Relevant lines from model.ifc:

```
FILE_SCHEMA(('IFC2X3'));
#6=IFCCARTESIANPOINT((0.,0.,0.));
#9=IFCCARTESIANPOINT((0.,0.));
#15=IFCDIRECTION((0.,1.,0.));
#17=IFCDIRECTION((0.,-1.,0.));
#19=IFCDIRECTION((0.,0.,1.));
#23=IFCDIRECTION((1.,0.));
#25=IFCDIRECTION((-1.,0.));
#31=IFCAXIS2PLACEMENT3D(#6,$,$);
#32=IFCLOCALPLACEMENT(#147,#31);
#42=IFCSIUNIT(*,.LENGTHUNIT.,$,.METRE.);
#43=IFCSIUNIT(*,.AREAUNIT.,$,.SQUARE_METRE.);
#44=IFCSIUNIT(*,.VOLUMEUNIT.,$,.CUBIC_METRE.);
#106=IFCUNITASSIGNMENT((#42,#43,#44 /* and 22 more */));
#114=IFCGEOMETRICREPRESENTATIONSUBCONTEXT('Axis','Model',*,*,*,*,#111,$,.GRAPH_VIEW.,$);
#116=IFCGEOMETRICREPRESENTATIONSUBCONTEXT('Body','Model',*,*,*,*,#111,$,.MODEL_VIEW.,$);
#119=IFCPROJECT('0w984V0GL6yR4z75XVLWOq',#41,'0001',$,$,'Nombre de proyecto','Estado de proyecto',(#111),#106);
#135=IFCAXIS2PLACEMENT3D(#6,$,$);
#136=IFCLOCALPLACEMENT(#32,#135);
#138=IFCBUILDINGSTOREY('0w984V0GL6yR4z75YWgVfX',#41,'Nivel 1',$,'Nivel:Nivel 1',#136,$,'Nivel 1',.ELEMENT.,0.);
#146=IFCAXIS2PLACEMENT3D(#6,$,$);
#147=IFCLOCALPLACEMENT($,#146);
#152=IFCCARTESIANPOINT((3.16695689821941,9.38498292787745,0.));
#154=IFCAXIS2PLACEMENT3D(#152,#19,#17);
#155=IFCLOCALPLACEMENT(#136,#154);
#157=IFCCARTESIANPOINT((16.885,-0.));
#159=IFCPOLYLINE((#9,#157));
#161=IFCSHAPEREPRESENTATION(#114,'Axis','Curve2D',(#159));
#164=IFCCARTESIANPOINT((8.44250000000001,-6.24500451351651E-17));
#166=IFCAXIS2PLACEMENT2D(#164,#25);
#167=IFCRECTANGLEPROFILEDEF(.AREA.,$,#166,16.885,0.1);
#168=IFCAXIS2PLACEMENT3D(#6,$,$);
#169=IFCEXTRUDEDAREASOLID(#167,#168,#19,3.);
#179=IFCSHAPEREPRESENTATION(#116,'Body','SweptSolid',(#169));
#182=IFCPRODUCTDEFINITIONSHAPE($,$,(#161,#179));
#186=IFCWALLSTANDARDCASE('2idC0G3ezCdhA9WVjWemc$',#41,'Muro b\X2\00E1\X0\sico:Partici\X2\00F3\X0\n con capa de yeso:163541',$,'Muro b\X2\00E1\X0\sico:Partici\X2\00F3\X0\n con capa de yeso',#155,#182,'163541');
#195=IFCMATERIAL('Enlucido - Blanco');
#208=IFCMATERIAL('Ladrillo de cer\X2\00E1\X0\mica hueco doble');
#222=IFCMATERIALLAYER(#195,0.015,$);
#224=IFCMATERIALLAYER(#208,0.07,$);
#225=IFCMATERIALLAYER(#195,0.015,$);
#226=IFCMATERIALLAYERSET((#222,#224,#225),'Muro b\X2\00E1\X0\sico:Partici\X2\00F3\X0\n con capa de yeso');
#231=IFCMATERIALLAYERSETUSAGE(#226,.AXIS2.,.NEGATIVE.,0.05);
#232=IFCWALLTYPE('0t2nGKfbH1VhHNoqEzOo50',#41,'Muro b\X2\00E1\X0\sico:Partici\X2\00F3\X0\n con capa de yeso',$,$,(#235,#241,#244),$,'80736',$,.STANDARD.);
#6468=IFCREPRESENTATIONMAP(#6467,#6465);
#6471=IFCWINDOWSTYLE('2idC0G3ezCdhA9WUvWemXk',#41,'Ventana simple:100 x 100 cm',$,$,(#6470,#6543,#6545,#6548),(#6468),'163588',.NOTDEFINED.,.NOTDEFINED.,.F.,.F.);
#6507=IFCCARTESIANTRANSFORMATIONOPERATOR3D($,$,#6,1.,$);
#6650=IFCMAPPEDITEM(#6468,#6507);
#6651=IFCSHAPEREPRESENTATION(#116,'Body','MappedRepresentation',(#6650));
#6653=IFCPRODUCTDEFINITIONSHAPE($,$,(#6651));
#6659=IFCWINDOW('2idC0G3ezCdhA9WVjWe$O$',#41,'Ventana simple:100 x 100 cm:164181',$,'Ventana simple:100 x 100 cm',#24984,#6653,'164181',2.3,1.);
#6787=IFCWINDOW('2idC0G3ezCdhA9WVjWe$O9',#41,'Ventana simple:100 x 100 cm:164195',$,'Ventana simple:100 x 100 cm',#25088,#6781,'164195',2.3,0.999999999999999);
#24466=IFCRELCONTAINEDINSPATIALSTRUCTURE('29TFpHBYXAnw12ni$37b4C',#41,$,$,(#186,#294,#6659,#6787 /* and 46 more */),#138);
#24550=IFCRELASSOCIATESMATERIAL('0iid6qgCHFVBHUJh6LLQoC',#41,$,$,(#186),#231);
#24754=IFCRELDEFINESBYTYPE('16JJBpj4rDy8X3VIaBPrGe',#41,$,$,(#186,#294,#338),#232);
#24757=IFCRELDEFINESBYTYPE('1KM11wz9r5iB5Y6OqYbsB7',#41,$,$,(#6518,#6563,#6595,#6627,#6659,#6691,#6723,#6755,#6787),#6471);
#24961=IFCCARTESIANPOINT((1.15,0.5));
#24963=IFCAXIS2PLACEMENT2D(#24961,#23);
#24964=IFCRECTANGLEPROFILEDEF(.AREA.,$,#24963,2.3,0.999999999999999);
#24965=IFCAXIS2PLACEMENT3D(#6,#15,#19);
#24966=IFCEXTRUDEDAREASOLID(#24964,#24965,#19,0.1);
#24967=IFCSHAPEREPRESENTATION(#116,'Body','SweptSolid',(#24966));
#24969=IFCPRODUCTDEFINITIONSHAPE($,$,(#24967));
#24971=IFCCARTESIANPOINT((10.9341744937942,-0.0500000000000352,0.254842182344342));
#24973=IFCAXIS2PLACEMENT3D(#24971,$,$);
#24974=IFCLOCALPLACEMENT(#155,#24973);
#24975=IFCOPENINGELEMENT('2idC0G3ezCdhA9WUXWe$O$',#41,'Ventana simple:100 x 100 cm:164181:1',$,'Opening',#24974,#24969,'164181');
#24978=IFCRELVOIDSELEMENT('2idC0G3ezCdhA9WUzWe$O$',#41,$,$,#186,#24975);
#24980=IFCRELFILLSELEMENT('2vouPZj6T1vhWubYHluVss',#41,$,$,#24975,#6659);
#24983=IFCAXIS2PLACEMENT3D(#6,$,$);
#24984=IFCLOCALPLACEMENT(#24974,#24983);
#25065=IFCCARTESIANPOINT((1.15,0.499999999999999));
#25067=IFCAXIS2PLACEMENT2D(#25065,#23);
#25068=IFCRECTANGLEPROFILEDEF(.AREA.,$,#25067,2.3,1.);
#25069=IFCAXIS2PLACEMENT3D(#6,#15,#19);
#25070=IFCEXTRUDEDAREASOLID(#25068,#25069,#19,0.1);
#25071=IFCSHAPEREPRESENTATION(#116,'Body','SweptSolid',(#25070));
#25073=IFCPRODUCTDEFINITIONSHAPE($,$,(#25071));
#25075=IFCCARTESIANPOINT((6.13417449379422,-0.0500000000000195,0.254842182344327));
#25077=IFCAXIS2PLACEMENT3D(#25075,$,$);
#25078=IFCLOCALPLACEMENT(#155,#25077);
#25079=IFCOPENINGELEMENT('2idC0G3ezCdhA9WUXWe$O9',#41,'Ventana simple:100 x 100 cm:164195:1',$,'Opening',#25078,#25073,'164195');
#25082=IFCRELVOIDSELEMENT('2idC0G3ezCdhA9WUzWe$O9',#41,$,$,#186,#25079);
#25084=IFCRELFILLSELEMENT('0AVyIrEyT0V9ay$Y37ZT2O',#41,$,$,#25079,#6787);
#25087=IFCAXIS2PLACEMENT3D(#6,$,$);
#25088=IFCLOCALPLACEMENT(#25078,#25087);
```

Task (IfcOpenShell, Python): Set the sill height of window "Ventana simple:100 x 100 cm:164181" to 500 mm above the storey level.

```python
import numpy as np
import ifcopenshell
import ifcopenshell.api.geometry
import ifcopenshell.geom
import ifcopenshell.util.element
import ifcopenshell.util.placement
import ifcopenshell.util.shape
import ifcopenshell.util.unit

model = ifcopenshell.open("model.ifc")
unit_scale = ifcopenshell.util.unit.calculate_unit_scale(model)

window = model.by_guid("2idC0G3ezCdhA9WVjWe$O$")
opening = window.FillsVoids[0].RelatingOpeningElement
storey = ifcopenshell.util.element.get_container(window, ifc_class="IfcBuildingStorey")
level = ifcopenshell.util.placement.get_local_placement(storey.ObjectPlacement)[2, 3]

# The opening's origin need not be at the sill, so measure its lowest point.
shape = ifcopenshell.geom.create_shape(ifcopenshell.geom.settings(), opening)
bottom = ifcopenshell.util.shape.get_shape_bottom_elevation(shape, shape.geometry) / unit_scale
dz = level + 0.5 - bottom

shift = np.array([0.0, 0.0, dz])
# The window is placed relative to its opening, so it follows when the opening moves.
matrix = ifcopenshell.util.placement.get_local_placement(opening.ObjectPlacement)
matrix[:3, 3] += shift
ifcopenshell.api.geometry.edit_object_placement(
    model, product=opening, matrix=matrix, is_si=False, should_transform_children=True
)

print(f"moved by {dz * unit_scale:+.3f} m")

model.write("model_rev.ifc")
```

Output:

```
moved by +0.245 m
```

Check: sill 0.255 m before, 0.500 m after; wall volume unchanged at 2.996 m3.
